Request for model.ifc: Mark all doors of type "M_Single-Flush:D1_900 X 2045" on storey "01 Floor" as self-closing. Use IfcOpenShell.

First a look at what the model holds.

```python
import ifcopenshell
import ifcopenshell.util.element

model = ifcopenshell.open("model.ifc")
print(model.schema)
storey = next(s for s in model.by_type("IfcBuildingStorey") if s.Name == "01 Floor")
doors = [e for e in ifcopenshell.util.element.get_decomposition(storey) if e.is_a("IfcDoor")]
seen = {}
for e in doors:
    element_type = ifcopenshell.util.element.get_type(e)
    key = (element_type.Name if element_type != e and element_type else None, ifcopenshell.util.element.get_pset(e, "Pset_DoorCommon", "SelfClosing"))
    seen[key] = seen.get(key, 0) + 1
for (name, value), count in sorted(seen.items(), key=str):
    print(count, "x", name, "|", value)
```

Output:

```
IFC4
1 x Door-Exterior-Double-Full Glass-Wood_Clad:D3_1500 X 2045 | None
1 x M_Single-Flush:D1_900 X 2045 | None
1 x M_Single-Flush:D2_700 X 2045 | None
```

```python
import ifcopenshell
import ifcopenshell.api.pset
import ifcopenshell.util.element

model = ifcopenshell.open("model.ifc")

storey = next(s for s in model.by_type("IfcBuildingStorey") if s.Name == "01 Floor")
doors = [e for e in ifcopenshell.util.element.get_decomposition(storey) if e.is_a("IfcDoor")]

count = 0
for e in doors:
    element_type = ifcopenshell.util.element.get_type(e)
    if element_type in (None, e) or element_type.Name != "M_Single-Flush:D1_900 X 2045":
        continue
    # add_pset returns the element's existing set when there is one.
    pset = ifcopenshell.api.pset.add_pset(model, product=e, name="Pset_DoorCommon")
    ifcopenshell.api.pset.edit_pset(model, pset=pset, properties={"SelfClosing": True})
    count += 1

print(count, "doors updated")

model.write("model_rev.ifc")
```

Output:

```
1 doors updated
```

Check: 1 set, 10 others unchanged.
